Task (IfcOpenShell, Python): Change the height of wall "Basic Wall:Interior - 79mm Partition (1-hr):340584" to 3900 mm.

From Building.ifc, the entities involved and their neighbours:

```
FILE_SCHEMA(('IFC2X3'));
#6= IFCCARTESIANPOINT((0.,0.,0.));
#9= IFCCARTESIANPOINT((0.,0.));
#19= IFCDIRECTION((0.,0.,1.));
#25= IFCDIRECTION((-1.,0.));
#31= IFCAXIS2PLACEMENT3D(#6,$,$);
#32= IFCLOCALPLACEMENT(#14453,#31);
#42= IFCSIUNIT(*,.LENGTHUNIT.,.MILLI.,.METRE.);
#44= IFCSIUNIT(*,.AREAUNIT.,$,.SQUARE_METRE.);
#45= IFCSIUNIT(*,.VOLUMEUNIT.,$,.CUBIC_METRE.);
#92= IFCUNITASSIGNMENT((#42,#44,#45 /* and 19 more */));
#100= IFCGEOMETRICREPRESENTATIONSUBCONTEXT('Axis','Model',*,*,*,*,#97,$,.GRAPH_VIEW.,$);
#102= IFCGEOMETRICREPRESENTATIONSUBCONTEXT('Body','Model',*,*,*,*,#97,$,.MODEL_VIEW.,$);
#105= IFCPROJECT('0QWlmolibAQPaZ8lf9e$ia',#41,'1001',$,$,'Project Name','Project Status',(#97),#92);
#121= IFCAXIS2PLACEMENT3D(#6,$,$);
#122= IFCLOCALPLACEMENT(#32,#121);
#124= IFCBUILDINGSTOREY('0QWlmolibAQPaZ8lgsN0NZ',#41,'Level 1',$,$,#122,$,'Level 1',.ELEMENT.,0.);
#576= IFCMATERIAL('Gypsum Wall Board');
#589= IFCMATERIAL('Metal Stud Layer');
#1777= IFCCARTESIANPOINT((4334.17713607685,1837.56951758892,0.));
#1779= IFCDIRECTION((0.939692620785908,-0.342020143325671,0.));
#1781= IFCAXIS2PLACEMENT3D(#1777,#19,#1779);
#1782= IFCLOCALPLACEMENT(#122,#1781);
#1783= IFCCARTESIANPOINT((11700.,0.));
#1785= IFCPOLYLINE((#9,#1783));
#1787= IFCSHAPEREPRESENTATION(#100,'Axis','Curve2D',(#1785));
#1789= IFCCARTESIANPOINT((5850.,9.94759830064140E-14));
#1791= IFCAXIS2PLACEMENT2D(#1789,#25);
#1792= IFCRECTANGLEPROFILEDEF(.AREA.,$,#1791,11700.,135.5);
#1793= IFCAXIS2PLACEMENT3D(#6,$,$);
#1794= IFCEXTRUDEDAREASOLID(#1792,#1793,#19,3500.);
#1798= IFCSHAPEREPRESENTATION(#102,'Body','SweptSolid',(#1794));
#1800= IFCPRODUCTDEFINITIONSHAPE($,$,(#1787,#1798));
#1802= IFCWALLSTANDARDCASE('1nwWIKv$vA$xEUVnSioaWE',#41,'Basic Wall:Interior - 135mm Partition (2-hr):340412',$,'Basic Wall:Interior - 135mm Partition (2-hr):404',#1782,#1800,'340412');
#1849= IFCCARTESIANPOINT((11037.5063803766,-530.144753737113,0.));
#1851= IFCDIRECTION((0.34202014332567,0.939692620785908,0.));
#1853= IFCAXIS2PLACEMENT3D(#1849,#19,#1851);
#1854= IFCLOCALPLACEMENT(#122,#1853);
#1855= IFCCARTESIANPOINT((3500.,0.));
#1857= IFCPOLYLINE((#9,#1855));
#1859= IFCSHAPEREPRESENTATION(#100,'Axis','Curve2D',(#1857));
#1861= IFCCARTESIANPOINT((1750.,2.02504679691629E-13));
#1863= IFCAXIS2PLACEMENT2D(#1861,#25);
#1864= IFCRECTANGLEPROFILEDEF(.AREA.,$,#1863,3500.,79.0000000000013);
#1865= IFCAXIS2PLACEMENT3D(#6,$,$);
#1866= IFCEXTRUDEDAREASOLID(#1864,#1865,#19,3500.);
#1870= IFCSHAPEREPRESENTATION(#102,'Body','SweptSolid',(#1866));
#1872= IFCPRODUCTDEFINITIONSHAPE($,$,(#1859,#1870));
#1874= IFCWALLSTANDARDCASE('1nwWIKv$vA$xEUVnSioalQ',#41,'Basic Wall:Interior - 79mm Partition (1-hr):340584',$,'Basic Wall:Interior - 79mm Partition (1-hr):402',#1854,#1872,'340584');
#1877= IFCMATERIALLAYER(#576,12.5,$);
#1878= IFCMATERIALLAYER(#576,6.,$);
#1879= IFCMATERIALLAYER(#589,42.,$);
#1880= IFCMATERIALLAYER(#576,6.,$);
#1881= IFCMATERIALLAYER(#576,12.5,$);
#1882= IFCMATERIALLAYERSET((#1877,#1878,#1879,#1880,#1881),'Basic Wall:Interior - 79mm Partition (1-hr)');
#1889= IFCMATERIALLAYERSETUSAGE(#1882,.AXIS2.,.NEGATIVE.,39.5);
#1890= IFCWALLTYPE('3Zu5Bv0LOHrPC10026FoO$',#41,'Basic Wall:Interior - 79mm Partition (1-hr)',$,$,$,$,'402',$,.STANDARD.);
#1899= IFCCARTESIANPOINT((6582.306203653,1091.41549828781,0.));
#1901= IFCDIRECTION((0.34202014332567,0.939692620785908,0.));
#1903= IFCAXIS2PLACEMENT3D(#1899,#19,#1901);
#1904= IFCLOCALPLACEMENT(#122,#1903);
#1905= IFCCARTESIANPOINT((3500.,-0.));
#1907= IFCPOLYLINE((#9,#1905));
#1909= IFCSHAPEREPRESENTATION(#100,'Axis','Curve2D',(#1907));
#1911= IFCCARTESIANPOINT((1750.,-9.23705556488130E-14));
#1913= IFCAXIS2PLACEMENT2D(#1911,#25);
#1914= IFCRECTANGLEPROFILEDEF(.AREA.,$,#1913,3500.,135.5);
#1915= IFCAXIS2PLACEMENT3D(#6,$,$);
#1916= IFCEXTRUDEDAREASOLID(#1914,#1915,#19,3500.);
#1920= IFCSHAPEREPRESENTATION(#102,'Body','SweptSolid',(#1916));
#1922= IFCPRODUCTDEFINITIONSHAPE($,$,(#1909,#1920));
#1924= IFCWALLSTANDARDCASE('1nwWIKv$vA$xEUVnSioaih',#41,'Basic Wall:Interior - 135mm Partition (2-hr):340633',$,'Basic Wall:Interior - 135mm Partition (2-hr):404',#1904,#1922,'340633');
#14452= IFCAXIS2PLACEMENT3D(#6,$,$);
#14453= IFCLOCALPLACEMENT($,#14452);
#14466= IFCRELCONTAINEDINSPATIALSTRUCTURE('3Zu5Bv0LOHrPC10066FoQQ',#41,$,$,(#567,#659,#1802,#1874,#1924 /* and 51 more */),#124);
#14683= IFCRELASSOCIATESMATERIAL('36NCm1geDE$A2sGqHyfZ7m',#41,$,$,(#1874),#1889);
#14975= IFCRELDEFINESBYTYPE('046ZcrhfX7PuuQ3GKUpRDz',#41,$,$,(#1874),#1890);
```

```python
import ifcopenshell
import ifcopenshell.geom
import ifcopenshell.util.representation
import ifcopenshell.util.shape

model = ifcopenshell.open("Building.ifc")
settings = ifcopenshell.geom.settings()


def volume(element):
    """Net volume in cubic metres, openings subtracted."""
    shape = ifcopenshell.geom.create_shape(settings, element)
    return ifcopenshell.util.shape.get_volume(shape.geometry)


wall = model.by_id(1874)
before = volume(wall)

body = ifcopenshell.util.representation.get_representation(wall, "Model", "Body")
solid = body.Items[0]
old_height = solid.Depth
solid.Depth = 3900.0
after = volume(wall)

print(f"height {old_height:g} -> {solid.Depth:g}, volume {before:.3f} -> {after:.3f} m3")

model.write("Building_updated.ifc")
```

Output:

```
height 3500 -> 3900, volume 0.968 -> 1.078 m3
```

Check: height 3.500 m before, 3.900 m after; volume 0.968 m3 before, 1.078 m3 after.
